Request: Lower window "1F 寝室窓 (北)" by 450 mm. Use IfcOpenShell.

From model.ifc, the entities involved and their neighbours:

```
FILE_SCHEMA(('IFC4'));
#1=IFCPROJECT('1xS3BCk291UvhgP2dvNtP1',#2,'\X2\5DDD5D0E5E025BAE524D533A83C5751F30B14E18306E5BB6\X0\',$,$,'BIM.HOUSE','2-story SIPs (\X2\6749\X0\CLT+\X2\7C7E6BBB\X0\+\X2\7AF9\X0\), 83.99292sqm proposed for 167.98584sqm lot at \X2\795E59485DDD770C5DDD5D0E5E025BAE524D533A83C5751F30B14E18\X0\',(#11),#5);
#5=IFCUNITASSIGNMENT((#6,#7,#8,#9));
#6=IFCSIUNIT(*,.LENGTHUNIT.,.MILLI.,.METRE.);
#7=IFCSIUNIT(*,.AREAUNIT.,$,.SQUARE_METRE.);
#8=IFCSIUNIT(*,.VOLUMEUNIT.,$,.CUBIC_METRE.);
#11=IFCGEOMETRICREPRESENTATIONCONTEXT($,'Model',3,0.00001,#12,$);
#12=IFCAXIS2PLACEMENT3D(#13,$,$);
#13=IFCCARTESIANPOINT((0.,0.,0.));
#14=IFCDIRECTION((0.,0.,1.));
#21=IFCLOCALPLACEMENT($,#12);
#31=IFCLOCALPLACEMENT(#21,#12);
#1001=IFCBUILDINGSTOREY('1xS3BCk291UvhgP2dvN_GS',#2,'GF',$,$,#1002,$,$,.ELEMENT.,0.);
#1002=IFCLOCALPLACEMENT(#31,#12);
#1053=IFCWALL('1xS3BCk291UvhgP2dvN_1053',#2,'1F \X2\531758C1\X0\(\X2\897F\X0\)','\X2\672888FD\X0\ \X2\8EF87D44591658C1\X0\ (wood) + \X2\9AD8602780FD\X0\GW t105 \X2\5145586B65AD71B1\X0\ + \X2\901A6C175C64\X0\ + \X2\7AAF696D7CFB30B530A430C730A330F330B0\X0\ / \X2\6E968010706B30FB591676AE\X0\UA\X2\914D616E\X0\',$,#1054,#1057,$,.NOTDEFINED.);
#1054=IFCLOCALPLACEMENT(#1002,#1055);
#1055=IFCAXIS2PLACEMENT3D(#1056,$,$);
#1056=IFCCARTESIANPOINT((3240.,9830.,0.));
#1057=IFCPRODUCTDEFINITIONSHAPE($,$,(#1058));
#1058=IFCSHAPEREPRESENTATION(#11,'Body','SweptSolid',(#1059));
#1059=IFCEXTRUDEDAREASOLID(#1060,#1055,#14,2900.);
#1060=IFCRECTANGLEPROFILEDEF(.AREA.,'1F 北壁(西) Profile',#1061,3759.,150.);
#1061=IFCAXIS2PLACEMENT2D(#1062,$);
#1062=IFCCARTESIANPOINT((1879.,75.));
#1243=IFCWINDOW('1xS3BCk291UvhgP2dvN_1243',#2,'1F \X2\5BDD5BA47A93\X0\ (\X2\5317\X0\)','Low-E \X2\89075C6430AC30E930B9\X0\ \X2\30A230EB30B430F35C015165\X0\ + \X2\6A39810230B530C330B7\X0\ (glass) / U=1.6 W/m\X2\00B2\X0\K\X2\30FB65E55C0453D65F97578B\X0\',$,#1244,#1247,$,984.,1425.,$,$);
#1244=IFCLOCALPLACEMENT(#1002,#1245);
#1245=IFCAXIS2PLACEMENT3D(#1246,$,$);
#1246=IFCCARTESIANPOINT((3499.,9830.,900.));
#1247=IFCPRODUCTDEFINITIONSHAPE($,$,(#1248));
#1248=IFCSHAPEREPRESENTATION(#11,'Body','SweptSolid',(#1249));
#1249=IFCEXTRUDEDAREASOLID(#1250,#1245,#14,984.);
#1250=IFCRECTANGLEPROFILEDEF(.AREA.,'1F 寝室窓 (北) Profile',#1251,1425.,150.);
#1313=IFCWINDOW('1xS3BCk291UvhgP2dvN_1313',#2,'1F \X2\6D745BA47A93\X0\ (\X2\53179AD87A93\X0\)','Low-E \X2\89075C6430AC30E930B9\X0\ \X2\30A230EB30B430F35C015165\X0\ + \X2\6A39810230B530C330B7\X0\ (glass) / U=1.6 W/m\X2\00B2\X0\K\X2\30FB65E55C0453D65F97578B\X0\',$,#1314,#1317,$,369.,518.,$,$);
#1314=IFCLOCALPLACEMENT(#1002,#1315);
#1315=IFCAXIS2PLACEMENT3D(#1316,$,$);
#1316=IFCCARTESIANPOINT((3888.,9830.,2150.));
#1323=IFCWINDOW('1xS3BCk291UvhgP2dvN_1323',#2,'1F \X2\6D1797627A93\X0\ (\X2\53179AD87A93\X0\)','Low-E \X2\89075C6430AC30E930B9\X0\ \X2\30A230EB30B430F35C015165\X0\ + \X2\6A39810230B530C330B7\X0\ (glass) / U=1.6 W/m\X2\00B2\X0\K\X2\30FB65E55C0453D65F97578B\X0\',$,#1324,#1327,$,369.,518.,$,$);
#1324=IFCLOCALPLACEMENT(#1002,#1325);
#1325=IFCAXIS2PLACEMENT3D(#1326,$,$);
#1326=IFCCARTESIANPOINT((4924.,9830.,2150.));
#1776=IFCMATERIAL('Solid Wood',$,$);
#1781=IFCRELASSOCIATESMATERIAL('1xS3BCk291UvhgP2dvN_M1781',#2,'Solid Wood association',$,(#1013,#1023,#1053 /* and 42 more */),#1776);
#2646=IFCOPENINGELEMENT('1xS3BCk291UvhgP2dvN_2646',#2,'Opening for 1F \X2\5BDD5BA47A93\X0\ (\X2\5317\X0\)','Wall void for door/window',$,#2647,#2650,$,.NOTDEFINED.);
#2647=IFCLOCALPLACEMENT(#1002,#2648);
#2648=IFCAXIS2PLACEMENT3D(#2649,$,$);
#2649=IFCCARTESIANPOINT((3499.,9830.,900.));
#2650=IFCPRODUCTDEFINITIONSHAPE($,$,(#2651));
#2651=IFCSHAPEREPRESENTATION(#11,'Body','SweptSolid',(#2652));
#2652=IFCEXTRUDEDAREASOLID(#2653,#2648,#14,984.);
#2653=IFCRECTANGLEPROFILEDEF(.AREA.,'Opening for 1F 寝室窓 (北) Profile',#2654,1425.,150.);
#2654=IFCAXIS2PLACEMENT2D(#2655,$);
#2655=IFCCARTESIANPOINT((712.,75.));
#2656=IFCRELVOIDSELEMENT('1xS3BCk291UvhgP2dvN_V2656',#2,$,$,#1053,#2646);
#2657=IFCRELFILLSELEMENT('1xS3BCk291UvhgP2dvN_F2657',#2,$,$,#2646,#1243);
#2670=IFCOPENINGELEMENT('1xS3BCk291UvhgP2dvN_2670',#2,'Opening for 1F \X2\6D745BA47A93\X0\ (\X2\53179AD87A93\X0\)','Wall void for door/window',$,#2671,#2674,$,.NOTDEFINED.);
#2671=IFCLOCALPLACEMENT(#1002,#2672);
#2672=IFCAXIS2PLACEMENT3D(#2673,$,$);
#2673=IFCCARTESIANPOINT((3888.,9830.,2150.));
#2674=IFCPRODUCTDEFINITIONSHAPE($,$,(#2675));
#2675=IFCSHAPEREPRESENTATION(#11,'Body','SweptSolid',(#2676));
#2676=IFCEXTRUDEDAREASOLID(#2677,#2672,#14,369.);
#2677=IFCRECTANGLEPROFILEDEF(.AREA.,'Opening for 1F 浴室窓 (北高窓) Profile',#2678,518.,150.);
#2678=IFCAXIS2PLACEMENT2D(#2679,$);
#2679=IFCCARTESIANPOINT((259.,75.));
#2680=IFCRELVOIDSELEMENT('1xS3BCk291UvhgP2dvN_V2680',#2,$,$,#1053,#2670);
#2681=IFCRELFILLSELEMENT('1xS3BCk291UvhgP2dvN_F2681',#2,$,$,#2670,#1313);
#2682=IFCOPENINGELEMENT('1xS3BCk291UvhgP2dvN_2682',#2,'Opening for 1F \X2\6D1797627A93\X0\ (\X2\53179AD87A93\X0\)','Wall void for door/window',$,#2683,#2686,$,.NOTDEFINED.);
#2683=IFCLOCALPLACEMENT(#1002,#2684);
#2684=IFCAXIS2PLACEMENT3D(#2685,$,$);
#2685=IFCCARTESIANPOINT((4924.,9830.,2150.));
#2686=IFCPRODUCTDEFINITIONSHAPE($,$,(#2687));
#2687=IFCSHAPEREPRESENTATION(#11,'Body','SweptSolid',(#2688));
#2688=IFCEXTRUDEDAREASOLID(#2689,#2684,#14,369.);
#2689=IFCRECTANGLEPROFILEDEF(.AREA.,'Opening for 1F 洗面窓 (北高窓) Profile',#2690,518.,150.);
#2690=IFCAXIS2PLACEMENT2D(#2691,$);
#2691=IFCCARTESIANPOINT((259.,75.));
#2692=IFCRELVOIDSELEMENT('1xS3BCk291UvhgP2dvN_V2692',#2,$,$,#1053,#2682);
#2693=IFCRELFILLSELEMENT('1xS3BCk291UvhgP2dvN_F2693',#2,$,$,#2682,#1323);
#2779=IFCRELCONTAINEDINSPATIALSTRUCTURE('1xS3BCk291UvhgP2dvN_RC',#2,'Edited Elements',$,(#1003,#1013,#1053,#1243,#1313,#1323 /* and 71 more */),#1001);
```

```python
import numpy as np
import ifcopenshell
import ifcopenshell.api.geometry
import ifcopenshell.util.placement
import ifcopenshell.util.unit

model = ifcopenshell.open("model.ifc")
unit_scale = ifcopenshell.util.unit.calculate_unit_scale(model)

window = model.by_guid("1xS3BCk291UvhgP2dvN_1243")
opening = window.FillsVoids[0].RelatingOpeningElement
dz = -450.0

shift = np.array([0.0, 0.0, dz])
# The window is not placed relative to its opening, so move both.
for product in (opening, window):
    matrix = ifcopenshell.util.placement.get_local_placement(product.ObjectPlacement)
    matrix[:3, 3] += shift
    ifcopenshell.api.geometry.edit_object_placement(model, product=product, matrix=matrix, is_si=False)

print(f"moved by {dz * unit_scale:+.3f} m")

model.write("model_updated.ifc")
```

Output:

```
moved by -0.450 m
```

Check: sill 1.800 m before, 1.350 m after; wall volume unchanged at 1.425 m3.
